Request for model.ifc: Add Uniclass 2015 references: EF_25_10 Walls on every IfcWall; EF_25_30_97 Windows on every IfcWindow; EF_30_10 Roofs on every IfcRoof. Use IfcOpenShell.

First a look at what the model holds.

```python
import ifcopenshell

model = ifcopenshell.open("model.ifc")
print(model.schema)
print("classifications:", [c.Name for c in model.by_type("IfcClassification")])
for ifc_class in ("IfcDoor", "IfcRoof", "IfcStair", "IfcWall", "IfcWindow"):
    print(ifc_class, len(model.by_type(ifc_class)))
```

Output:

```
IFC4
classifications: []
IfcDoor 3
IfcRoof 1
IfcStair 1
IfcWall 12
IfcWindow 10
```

```python
import ifcopenshell
import ifcopenshell.api.classification

model = ifcopenshell.open("model.ifc")

system = ifcopenshell.api.classification.add_classification(model, classification="Uniclass 2015")

codes = {
    "IfcWall": ("EF_25_10", "Walls"),
    "IfcWindow": ("EF_25_30_97", "Windows"),
    "IfcRoof": ("EF_30_10", "Roofs"),
}
for ifc_class, (code, name) in codes.items():
    products = model.by_type(ifc_class)
    ifcopenshell.api.classification.add_reference(
        model, products=products, classification=system, identification=code, name=name
    )
    print(code, len(products))

model.write("model-out.ifc")
```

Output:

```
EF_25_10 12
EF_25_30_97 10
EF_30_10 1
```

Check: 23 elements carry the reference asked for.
